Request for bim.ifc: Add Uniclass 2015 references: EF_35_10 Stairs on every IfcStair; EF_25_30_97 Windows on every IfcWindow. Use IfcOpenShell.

First a look at what the model holds.

```python
import ifcopenshell

model = ifcopenshell.open("bim.ifc")
print(model.schema)
print("classifications:", [c.Name for c in model.by_type("IfcClassification")])
for ifc_class in ("IfcDoor", "IfcRoof", "IfcStair", "IfcWall", "IfcWindow"):
    print(ifc_class, len(model.by_type(ifc_class)))
```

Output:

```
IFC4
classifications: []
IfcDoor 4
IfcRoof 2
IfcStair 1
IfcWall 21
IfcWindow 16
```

```python
import ifcopenshell
import ifcopenshell.api.classification

model = ifcopenshell.open("bim.ifc")

system = ifcopenshell.api.classification.add_classification(model, classification="Uniclass 2015")

codes = {
    "IfcStair": ("EF_35_10", "Stairs"),
    "IfcWindow": ("EF_25_30_97", "Windows"),
}
for ifc_class, (code, name) in codes.items():
    products = model.by_type(ifc_class)
    ifcopenshell.api.classification.add_reference(
        model, products=products, classification=system, identification=code, name=name
    )
    print(code, len(products))

model.write("bim_edited.ifc")
```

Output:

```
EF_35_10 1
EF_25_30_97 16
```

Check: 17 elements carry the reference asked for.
